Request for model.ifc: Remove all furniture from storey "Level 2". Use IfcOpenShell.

First a look at what the model holds.

```python
import ifcopenshell
import ifcopenshell.util.element

model = ifcopenshell.open("model.ifc")
print(model.schema)
storey = next(s for s in model.by_type("IfcBuildingStorey") if s.Name == "Level 2")
furniture = [e for e in ifcopenshell.util.element.get_decomposition(storey) if e.is_a("IfcFurnishingElement")]
seen = {}
for e in furniture:
    element_type = ifcopenshell.util.element.get_type(e)
    name = element_type.Name if element_type not in (None, e) else None
    seen[name] = seen.get(name, 0) + 1
for name, count in sorted(seen.items(), key=str):
    print(count, "x", name)
```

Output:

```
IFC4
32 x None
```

```python
import ifcopenshell
import ifcopenshell.api.root
import ifcopenshell.util.element

model = ifcopenshell.open("model.ifc")

storey = next(s for s in model.by_type("IfcBuildingStorey") if s.Name == "Level 2")
furniture = [e for e in ifcopenshell.util.element.get_decomposition(storey) if e.is_a("IfcFurnishingElement")]

for e in furniture:
    ifcopenshell.api.root.remove_product(model, product=e)
print(len(furniture), "removed")

model.write("model_v2.ifc")
```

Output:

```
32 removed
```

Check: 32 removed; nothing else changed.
